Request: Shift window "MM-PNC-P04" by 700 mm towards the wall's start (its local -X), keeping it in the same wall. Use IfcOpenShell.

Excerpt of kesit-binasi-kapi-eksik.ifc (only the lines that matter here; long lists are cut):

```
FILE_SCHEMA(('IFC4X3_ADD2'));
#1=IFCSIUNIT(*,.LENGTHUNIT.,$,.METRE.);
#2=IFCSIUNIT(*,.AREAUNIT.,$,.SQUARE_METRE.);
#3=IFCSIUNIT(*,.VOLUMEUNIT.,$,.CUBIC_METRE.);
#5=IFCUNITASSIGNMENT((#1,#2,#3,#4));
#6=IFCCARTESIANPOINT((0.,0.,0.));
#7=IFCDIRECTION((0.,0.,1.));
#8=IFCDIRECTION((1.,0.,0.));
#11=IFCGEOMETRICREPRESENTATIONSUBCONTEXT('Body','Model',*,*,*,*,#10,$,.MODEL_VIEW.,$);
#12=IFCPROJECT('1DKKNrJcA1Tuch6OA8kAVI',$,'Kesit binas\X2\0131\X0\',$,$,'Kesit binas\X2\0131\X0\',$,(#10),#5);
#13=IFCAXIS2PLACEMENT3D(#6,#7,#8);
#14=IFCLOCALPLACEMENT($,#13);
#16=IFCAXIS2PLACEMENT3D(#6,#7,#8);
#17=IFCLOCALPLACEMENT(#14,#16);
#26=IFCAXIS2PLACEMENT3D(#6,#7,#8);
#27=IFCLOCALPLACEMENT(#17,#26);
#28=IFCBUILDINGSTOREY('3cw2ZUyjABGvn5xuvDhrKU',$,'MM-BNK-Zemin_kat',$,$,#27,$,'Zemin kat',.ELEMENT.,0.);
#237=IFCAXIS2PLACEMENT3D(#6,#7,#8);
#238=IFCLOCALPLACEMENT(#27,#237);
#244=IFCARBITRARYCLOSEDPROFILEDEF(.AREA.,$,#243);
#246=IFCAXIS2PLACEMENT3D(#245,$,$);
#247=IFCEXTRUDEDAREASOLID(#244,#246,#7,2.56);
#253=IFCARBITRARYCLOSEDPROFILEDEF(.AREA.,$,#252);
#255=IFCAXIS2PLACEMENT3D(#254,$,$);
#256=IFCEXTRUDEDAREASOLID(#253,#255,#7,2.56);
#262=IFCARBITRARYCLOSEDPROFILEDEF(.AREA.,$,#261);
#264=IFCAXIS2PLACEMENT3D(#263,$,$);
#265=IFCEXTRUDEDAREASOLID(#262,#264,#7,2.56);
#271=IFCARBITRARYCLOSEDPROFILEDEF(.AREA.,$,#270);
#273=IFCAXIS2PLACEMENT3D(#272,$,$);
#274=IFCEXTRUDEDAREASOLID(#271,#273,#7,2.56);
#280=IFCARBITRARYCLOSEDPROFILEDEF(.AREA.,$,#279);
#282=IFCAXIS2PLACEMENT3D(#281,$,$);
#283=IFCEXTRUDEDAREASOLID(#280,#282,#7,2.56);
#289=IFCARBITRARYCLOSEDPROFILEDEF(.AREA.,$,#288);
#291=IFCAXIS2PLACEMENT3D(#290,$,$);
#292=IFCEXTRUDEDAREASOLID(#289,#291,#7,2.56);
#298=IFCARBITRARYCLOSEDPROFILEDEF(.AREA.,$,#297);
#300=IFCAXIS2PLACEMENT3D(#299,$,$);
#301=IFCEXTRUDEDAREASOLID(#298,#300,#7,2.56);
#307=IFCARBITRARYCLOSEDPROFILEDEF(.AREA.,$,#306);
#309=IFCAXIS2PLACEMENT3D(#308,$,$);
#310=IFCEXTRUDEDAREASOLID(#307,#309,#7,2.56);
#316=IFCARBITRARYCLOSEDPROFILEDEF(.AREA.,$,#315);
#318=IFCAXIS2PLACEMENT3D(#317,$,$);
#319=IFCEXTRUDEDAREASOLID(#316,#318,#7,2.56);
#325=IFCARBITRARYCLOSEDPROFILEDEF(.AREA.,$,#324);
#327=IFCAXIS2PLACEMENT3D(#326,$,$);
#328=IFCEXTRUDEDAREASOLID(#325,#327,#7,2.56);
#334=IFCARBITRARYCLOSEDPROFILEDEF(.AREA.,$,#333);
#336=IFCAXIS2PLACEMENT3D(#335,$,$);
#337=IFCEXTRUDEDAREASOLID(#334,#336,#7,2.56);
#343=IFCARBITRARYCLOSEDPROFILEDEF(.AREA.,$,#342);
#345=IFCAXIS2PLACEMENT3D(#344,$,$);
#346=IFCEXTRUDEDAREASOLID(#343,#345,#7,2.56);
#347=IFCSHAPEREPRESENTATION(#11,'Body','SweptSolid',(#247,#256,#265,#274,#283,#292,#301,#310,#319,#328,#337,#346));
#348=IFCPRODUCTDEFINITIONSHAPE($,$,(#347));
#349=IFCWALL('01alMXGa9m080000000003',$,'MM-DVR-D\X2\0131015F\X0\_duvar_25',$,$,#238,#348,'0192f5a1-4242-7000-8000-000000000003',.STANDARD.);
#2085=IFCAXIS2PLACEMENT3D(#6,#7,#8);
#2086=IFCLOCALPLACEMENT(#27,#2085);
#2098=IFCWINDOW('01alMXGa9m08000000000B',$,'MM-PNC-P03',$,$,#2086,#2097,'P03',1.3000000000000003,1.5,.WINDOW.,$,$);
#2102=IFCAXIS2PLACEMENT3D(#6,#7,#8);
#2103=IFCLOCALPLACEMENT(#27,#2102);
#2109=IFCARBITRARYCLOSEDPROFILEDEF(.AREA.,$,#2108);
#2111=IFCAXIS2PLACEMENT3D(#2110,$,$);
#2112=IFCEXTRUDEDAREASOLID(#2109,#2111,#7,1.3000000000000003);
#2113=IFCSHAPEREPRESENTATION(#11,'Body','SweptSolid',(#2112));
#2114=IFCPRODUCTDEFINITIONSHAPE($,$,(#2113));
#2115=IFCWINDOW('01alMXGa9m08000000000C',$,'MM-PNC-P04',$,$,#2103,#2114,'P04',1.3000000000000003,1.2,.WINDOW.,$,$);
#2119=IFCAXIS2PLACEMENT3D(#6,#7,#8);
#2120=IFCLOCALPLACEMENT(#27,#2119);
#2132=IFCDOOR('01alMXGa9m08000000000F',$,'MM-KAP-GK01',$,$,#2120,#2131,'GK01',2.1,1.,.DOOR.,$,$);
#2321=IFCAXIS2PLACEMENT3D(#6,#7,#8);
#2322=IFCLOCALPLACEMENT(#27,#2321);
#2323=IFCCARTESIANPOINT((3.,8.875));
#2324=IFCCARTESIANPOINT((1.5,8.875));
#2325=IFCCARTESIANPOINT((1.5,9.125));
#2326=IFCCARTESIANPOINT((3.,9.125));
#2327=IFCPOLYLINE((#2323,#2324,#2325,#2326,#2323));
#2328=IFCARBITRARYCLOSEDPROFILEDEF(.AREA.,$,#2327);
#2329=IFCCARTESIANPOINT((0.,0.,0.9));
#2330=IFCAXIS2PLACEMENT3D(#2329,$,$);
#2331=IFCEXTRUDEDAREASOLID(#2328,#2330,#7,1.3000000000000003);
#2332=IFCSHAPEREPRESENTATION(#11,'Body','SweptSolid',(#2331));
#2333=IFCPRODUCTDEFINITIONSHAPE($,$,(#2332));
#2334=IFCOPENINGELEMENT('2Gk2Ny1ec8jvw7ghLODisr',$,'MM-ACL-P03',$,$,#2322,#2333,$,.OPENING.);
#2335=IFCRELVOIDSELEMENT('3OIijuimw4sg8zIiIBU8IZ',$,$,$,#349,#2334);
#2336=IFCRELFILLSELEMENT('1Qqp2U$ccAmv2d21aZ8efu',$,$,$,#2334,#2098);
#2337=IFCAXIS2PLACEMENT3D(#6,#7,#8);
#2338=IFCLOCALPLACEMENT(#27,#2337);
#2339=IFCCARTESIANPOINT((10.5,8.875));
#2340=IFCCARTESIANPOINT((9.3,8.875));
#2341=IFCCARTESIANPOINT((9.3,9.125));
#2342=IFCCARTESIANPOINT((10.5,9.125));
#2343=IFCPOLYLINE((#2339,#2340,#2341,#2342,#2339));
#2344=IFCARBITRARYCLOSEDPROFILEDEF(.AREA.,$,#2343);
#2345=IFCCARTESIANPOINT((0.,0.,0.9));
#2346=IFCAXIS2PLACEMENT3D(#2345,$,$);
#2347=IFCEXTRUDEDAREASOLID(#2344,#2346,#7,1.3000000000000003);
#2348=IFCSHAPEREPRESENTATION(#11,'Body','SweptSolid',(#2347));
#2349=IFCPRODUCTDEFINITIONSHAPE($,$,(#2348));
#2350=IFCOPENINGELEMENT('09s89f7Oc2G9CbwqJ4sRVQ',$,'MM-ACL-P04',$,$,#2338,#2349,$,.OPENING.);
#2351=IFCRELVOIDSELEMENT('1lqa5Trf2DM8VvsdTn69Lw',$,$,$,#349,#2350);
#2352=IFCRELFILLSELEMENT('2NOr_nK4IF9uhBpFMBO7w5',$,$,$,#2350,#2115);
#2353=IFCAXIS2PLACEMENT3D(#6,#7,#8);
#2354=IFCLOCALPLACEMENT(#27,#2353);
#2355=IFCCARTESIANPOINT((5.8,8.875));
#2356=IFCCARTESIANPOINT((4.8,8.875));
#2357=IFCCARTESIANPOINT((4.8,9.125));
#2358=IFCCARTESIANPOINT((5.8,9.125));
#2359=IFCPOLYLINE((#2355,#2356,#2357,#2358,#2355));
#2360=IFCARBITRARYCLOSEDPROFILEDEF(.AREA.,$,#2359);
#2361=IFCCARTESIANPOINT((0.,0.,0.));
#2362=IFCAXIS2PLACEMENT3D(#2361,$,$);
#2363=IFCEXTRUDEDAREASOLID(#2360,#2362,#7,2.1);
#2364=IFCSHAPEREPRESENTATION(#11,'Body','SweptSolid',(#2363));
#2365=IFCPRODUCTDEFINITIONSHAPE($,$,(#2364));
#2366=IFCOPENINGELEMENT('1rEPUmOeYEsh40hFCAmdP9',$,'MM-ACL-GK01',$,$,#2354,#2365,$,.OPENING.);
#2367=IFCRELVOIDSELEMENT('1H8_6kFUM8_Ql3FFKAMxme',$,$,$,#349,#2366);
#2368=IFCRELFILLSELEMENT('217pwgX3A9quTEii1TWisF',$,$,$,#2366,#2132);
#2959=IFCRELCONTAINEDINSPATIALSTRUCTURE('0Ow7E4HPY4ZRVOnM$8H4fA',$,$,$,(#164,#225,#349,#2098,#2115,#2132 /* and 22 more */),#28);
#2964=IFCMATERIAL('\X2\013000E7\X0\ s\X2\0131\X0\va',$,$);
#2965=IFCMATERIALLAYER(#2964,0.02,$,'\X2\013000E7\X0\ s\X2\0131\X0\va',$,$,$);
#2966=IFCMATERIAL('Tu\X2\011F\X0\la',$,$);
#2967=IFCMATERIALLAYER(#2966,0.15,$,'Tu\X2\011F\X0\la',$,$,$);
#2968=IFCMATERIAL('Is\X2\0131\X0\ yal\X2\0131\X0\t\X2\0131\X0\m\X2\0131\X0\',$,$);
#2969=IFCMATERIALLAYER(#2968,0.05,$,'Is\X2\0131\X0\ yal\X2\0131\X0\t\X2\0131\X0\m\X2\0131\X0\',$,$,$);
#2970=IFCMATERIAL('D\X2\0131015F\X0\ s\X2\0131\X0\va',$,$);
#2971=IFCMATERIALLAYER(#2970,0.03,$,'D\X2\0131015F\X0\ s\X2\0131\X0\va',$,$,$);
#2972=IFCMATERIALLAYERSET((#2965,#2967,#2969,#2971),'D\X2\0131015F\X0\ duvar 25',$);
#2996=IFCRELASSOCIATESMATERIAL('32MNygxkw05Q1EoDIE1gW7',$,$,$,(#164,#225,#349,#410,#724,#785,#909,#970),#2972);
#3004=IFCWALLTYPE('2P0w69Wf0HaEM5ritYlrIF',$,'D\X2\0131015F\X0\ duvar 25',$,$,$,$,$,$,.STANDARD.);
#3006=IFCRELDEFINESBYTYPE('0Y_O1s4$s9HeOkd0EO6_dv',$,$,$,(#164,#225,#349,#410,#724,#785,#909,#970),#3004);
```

```python
import ifcopenshell
import ifcopenshell.api.geometry
import ifcopenshell.util.placement
import ifcopenshell.util.unit

model = ifcopenshell.open("kesit-binasi-kapi-eksik.ifc")
unit_scale = ifcopenshell.util.unit.calculate_unit_scale(model)

window = model.by_guid("01alMXGa9m08000000000C")
opening = window.FillsVoids[0].RelatingOpeningElement
wall = opening.VoidsElements[0].RelatingBuildingElement

wall_matrix = ifcopenshell.util.placement.get_local_placement(wall.ObjectPlacement)
shift = wall_matrix[:3, 0] * -0.7 / unit_scale
before = ifcopenshell.util.placement.get_local_placement(window.ObjectPlacement)[:3, 3].copy()

# The window is not placed relative to its opening, so move both.
for product in (opening, window):
    matrix = ifcopenshell.util.placement.get_local_placement(product.ObjectPlacement)
    matrix[:3, 3] += shift
    ifcopenshell.api.geometry.edit_object_placement(model, product=product, matrix=matrix, is_si=False)

after = ifcopenshell.util.placement.get_local_placement(window.ObjectPlacement)[:3, 3]
print("window moved by", (after - before).round(3) + 0.0)

model.write("kesit-binasi-kapi-eksik_v2.ifc")
```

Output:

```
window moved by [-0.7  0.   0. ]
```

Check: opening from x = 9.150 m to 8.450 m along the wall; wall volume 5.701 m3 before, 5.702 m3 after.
